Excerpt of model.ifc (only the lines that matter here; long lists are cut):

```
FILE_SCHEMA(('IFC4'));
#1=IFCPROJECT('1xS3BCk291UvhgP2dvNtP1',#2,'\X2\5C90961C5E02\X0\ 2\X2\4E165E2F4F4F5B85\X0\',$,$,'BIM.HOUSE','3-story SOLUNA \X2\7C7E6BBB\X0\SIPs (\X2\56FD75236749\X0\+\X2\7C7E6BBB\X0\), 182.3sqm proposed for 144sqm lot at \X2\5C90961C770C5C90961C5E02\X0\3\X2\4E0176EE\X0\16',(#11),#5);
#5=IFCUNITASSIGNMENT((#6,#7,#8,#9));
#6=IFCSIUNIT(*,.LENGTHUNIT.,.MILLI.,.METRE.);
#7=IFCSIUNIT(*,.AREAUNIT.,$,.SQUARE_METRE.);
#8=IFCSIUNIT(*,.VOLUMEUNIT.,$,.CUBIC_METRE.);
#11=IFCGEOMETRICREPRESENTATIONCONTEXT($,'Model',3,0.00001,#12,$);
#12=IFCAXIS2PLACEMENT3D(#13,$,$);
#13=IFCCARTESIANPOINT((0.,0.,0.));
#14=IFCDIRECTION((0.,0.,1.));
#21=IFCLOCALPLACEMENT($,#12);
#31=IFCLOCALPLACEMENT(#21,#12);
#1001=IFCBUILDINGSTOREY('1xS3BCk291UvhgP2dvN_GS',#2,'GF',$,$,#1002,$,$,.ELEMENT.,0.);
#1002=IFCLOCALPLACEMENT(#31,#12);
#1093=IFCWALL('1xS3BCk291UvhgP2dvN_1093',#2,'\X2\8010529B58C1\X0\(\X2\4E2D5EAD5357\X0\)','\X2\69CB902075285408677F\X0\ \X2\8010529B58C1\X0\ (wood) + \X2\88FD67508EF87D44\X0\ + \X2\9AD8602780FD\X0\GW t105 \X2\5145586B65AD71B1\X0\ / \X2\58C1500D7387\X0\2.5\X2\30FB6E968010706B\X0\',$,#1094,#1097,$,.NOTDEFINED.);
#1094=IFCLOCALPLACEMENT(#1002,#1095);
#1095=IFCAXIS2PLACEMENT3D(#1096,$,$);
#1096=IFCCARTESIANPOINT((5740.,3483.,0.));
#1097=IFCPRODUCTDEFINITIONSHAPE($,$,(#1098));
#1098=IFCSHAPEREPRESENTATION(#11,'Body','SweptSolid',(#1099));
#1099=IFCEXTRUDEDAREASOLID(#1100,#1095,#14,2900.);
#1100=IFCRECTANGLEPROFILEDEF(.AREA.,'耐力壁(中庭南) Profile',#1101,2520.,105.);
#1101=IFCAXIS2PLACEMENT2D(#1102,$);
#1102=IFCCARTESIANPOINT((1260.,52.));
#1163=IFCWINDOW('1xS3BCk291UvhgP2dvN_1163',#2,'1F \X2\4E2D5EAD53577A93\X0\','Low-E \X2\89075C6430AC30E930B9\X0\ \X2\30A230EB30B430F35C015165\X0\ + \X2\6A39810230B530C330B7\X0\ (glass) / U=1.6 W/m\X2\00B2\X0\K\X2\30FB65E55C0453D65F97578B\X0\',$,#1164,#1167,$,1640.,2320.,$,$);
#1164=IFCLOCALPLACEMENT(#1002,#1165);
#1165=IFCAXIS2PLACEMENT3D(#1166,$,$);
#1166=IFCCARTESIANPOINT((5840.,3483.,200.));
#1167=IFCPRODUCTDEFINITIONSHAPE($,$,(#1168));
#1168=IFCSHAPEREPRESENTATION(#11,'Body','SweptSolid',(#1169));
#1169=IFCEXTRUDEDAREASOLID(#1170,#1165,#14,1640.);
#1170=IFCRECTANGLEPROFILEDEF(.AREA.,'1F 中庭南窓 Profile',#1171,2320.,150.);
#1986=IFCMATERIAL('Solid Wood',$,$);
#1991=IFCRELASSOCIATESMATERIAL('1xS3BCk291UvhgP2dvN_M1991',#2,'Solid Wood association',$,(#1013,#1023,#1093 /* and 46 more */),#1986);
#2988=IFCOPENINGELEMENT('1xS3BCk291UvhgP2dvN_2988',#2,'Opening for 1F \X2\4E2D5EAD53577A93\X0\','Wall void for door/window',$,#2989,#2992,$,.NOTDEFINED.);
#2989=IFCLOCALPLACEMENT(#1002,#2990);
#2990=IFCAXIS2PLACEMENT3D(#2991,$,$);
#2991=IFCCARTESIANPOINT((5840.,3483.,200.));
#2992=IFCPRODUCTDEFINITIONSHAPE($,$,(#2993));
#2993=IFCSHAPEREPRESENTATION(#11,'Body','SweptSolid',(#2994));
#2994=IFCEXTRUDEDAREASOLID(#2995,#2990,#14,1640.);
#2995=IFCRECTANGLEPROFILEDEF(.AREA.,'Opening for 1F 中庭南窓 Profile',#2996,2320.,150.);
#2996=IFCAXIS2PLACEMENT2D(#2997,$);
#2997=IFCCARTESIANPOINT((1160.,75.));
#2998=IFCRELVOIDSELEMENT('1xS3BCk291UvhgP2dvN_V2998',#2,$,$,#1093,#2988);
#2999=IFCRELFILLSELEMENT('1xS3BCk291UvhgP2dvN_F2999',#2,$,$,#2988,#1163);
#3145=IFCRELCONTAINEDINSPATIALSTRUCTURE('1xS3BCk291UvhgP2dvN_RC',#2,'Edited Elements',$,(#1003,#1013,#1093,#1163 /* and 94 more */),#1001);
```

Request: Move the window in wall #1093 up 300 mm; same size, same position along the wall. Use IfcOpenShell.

```python
import numpy as np
import ifcopenshell
import ifcopenshell.api.geometry
import ifcopenshell.util.placement
import ifcopenshell.util.unit

model = ifcopenshell.open("model.ifc")
unit_scale = ifcopenshell.util.unit.calculate_unit_scale(model)

window = model.by_guid("1xS3BCk291UvhgP2dvN_1163")
opening = window.FillsVoids[0].RelatingOpeningElement
dz = 300.0

shift = np.array([0.0, 0.0, dz])
# The window is not placed relative to its opening, so move both.
for product in (opening, window):
    matrix = ifcopenshell.util.placement.get_local_placement(product.ObjectPlacement)
    matrix[:3, 3] += shift
    ifcopenshell.api.geometry.edit_object_placement(model, product=product, matrix=matrix, is_si=False)

print(f"moved by {dz * unit_scale:+.3f} m")

model.write("model_updated.ifc")
```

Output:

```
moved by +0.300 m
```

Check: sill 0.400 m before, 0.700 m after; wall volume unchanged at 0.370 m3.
